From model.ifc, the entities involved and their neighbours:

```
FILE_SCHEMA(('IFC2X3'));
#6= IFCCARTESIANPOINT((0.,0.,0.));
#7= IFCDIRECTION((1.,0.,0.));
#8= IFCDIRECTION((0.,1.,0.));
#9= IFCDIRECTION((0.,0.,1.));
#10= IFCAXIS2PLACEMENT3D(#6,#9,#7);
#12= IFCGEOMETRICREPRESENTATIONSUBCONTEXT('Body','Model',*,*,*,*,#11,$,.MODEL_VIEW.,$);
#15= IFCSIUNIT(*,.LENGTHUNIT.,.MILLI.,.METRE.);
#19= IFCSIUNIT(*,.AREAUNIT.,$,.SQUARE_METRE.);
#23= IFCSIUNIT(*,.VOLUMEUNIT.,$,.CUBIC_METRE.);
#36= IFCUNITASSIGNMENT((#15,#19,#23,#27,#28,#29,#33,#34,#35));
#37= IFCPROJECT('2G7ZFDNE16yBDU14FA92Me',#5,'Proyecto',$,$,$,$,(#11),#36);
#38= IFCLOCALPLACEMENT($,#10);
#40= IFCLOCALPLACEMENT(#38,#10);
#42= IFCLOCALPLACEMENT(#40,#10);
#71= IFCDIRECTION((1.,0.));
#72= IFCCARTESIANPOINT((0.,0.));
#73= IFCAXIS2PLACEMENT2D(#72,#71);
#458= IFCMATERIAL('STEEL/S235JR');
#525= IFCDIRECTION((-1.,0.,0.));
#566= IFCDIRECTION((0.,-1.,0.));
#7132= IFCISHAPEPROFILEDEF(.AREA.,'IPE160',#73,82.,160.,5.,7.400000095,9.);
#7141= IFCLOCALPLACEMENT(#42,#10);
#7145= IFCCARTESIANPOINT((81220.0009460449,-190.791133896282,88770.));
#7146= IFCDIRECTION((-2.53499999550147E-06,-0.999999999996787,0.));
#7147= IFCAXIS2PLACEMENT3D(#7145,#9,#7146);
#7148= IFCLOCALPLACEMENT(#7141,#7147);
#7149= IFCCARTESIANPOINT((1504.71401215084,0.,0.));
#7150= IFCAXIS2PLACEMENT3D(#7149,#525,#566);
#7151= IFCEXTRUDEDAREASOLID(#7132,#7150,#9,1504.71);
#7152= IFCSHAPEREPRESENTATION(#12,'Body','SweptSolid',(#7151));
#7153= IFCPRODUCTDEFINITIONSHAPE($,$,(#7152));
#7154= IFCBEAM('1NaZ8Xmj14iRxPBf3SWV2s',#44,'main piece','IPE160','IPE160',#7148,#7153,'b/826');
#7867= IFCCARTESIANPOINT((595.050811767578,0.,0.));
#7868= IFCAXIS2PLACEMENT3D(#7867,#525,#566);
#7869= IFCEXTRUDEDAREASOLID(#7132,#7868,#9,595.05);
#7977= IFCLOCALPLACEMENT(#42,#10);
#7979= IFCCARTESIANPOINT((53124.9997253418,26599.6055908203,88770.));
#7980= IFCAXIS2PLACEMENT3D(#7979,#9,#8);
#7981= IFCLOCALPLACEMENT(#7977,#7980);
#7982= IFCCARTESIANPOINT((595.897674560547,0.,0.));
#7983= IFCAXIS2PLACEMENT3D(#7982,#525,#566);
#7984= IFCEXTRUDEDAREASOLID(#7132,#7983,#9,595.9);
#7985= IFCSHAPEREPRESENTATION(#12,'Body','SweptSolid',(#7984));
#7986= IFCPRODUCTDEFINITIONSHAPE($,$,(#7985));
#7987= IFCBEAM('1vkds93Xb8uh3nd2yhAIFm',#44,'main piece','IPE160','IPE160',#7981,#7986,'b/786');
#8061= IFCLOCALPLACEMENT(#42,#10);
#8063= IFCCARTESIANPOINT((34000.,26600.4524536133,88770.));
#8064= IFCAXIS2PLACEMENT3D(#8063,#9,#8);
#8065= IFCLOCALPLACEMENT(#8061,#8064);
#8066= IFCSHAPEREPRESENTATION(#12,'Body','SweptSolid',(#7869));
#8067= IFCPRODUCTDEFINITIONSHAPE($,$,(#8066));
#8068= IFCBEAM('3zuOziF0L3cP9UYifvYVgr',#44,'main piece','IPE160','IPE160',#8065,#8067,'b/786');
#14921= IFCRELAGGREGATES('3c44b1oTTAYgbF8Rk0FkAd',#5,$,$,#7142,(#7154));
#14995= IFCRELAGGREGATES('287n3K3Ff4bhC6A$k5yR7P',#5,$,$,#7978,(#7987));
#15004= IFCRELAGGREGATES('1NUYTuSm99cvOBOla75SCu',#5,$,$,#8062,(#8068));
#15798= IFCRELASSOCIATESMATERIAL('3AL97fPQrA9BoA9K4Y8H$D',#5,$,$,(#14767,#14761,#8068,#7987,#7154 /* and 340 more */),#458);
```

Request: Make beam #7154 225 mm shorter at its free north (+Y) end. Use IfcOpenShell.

```python
import ifcopenshell
import ifcopenshell.util.representation
import ifcopenshell.util.unit

model = ifcopenshell.open("model.ifc")
unit_scale = ifcopenshell.util.unit.calculate_unit_scale(model)

member = model.by_guid("1NaZ8Xmj14iRxPBf3SWV2s")
change = -0.225 / unit_scale

# The extrusion runs towards the end named, so only its depth changes.
body = ifcopenshell.util.representation.get_representation(member, "Model", "Body")
solid = body.Items[0]
old_length = solid.Depth
solid.Depth += change

print(f"length {old_length:g} -> {solid.Depth:g}")

model.write("model_edited.ifc")
```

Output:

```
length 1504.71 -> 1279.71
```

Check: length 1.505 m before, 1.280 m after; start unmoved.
